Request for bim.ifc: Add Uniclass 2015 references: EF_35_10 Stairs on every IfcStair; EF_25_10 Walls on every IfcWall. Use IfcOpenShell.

First a look at what the model holds.

```python
import ifcopenshell

model = ifcopenshell.open("bim.ifc")
print(model.schema)
print("classifications:", [c.Name for c in model.by_type("IfcClassification")])
for ifc_class in ("IfcDoor", "IfcRoof", "IfcStair", "IfcWall", "IfcWindow"):
    print(ifc_class, len(model.by_type(ifc_class)))
```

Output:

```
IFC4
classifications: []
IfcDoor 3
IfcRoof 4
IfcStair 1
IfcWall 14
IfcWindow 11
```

```python
import ifcopenshell
import ifcopenshell.api.classification

model = ifcopenshell.open("bim.ifc")

system = ifcopenshell.api.classification.add_classification(model, classification="Uniclass 2015")

codes = {
    "IfcStair": ("EF_35_10", "Stairs"),
    "IfcWall": ("EF_25_10", "Walls"),
}
for ifc_class, (code, name) in codes.items():
    products = model.by_type(ifc_class)
    ifcopenshell.api.classification.add_reference(
        model, products=products, classification=system, identification=code, name=name
    )
    print(code, len(products))

model.write("bim_v2.ifc")
```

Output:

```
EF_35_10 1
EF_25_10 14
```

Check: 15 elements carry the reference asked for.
